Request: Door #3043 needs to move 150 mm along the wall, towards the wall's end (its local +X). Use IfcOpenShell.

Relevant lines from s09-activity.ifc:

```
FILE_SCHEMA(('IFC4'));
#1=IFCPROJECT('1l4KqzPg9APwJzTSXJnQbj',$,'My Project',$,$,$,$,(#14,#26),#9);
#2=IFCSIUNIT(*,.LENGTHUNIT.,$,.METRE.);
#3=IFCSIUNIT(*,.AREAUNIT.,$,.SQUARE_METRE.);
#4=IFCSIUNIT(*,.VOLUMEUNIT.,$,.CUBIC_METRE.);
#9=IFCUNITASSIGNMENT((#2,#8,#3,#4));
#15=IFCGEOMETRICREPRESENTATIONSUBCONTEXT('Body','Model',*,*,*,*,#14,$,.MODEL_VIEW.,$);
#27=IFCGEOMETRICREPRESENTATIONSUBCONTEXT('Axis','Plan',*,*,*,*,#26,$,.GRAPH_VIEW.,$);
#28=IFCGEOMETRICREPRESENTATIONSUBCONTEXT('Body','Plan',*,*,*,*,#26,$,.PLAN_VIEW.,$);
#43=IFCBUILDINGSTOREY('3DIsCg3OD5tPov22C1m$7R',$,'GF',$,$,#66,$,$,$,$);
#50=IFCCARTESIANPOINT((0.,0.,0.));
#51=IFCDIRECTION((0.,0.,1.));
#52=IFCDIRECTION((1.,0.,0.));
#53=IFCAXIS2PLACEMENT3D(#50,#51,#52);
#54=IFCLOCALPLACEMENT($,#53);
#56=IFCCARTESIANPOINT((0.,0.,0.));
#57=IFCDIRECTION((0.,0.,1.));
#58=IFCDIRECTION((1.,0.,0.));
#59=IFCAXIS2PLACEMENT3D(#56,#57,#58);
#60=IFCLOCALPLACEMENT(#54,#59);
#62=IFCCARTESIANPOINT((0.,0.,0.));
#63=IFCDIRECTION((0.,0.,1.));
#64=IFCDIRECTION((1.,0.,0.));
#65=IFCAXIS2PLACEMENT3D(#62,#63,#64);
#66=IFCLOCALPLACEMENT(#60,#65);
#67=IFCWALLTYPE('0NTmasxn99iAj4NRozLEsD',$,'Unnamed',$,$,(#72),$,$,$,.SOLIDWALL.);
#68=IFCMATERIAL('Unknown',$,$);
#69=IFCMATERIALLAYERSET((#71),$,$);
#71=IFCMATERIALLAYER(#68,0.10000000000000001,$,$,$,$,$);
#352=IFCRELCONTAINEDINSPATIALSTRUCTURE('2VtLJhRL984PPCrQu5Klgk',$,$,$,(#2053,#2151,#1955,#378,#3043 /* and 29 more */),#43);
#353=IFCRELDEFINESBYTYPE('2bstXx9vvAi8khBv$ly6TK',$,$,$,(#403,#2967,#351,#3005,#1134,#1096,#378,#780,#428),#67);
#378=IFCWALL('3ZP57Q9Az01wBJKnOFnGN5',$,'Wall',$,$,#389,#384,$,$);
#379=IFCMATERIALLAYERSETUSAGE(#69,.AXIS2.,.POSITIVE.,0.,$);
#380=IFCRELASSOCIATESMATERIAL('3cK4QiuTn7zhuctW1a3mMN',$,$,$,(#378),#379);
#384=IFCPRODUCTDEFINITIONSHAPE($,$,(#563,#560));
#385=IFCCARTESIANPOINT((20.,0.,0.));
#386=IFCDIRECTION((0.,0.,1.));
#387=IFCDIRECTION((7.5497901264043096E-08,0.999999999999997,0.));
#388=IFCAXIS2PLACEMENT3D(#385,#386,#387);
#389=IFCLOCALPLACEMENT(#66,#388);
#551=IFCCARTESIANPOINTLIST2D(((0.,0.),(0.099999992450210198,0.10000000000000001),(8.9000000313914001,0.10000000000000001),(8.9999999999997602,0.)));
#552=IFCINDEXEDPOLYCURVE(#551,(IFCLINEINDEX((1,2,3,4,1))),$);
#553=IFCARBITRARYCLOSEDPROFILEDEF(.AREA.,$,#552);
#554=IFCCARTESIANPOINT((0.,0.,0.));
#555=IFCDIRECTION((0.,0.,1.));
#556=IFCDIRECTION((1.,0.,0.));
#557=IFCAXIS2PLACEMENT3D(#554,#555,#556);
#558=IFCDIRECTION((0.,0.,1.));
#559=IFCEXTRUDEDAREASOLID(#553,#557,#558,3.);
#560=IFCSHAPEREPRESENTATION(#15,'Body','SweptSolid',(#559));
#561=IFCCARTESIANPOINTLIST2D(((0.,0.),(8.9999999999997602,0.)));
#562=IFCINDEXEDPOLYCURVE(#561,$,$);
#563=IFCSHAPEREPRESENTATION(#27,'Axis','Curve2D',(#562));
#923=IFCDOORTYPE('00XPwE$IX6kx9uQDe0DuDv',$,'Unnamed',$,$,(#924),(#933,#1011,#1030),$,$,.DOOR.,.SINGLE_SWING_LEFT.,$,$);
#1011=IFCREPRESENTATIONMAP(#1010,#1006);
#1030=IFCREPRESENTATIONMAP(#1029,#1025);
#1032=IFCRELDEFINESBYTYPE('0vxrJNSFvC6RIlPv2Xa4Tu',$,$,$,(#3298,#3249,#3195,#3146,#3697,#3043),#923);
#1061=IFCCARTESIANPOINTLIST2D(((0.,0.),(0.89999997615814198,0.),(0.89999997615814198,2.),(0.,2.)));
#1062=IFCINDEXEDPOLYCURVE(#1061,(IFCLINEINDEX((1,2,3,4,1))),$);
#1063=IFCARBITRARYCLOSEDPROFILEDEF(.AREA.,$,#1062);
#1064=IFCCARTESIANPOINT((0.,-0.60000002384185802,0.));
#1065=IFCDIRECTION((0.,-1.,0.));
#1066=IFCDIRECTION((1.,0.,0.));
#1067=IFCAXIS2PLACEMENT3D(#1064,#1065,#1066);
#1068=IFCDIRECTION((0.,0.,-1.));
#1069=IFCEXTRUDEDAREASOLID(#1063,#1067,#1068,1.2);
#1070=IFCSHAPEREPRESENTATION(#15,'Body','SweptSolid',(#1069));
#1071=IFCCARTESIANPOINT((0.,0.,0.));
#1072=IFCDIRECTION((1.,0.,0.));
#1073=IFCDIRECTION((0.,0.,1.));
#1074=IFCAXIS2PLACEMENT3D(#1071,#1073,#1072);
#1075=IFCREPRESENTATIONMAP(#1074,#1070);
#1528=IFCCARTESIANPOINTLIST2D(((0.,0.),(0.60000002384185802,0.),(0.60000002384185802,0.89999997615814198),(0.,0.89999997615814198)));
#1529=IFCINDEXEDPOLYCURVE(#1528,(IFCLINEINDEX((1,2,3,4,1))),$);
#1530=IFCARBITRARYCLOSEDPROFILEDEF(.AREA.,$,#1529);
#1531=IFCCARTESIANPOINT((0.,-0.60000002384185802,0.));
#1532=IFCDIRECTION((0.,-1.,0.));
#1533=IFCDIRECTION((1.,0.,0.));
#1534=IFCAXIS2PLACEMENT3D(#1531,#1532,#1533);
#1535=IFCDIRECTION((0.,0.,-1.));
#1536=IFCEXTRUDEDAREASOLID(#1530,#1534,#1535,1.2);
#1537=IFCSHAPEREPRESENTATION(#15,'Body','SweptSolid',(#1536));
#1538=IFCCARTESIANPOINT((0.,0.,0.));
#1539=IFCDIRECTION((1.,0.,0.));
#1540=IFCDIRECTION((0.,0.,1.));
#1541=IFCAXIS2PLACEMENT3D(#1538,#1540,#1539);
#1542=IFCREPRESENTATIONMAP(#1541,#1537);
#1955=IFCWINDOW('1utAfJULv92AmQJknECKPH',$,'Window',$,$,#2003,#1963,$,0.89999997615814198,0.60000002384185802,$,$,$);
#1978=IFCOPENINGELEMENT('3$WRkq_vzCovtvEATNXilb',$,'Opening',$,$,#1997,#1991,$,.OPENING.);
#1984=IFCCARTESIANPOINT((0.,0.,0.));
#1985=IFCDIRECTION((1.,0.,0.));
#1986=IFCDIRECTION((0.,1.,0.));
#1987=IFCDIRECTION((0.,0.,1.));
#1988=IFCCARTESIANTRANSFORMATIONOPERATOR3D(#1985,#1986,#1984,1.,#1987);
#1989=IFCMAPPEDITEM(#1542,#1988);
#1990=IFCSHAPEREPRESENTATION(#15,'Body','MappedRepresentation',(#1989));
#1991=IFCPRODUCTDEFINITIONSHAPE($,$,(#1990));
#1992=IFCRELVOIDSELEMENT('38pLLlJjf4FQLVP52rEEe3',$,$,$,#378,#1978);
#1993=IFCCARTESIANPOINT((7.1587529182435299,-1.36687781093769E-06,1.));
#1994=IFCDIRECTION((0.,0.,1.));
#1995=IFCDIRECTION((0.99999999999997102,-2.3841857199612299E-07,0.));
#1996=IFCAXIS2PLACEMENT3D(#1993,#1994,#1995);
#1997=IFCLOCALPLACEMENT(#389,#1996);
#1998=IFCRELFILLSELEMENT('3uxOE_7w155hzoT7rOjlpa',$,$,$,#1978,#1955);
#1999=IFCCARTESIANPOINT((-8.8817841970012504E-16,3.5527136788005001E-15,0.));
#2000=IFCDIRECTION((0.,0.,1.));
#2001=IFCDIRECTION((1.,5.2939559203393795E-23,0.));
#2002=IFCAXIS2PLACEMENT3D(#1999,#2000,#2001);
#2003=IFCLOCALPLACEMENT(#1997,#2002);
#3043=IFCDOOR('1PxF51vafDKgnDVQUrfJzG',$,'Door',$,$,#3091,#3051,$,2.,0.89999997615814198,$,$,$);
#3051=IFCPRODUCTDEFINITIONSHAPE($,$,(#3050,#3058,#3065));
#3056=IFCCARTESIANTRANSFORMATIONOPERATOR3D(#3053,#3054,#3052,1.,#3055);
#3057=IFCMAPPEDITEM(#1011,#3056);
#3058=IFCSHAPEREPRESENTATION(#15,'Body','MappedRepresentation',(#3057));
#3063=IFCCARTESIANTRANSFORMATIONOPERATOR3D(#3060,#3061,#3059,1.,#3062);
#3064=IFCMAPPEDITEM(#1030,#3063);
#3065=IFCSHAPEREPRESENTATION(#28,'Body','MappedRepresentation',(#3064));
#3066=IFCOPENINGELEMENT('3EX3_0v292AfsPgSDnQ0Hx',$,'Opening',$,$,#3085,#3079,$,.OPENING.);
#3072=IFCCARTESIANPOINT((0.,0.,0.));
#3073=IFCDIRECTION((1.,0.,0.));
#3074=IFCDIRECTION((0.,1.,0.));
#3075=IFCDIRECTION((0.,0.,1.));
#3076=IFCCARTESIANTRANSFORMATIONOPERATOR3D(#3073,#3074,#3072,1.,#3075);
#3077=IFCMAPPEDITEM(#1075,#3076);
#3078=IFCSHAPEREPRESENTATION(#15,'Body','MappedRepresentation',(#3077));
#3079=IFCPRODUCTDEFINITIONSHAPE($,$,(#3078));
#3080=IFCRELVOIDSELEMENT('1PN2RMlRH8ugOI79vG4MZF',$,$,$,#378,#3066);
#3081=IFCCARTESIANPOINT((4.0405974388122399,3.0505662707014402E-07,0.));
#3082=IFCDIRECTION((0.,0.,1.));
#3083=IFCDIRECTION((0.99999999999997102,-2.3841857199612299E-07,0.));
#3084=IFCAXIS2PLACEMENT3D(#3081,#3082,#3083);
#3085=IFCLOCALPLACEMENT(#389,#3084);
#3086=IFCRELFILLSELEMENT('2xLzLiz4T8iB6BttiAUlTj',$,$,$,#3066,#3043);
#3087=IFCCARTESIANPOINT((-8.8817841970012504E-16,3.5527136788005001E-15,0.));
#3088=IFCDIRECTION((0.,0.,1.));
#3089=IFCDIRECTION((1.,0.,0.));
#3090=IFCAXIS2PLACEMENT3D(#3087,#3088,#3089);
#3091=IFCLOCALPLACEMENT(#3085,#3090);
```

```python
import ifcopenshell
import ifcopenshell.api.geometry
import ifcopenshell.util.placement
import ifcopenshell.util.unit

model = ifcopenshell.open("s09-activity.ifc")
unit_scale = ifcopenshell.util.unit.calculate_unit_scale(model)

door = model.by_guid("1PxF51vafDKgnDVQUrfJzG")
opening = door.FillsVoids[0].RelatingOpeningElement
wall = opening.VoidsElements[0].RelatingBuildingElement

wall_matrix = ifcopenshell.util.placement.get_local_placement(wall.ObjectPlacement)
shift = wall_matrix[:3, 0] * 0.15 / unit_scale
before = ifcopenshell.util.placement.get_local_placement(door.ObjectPlacement)[:3, 3].copy()

# The door is placed relative to its opening, so it follows when the opening moves.
matrix = ifcopenshell.util.placement.get_local_placement(opening.ObjectPlacement)
matrix[:3, 3] += shift
ifcopenshell.api.geometry.edit_object_placement(
    model, product=opening, matrix=matrix, is_si=False, should_transform_children=True
)

after = ifcopenshell.util.placement.get_local_placement(door.ObjectPlacement)[:3, 3]
print("door moved by", (after - before).round(3) + 0.0)

model.write("s09-activity_v2.ifc")
```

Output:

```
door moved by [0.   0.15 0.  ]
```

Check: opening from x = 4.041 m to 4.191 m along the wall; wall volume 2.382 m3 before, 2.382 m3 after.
